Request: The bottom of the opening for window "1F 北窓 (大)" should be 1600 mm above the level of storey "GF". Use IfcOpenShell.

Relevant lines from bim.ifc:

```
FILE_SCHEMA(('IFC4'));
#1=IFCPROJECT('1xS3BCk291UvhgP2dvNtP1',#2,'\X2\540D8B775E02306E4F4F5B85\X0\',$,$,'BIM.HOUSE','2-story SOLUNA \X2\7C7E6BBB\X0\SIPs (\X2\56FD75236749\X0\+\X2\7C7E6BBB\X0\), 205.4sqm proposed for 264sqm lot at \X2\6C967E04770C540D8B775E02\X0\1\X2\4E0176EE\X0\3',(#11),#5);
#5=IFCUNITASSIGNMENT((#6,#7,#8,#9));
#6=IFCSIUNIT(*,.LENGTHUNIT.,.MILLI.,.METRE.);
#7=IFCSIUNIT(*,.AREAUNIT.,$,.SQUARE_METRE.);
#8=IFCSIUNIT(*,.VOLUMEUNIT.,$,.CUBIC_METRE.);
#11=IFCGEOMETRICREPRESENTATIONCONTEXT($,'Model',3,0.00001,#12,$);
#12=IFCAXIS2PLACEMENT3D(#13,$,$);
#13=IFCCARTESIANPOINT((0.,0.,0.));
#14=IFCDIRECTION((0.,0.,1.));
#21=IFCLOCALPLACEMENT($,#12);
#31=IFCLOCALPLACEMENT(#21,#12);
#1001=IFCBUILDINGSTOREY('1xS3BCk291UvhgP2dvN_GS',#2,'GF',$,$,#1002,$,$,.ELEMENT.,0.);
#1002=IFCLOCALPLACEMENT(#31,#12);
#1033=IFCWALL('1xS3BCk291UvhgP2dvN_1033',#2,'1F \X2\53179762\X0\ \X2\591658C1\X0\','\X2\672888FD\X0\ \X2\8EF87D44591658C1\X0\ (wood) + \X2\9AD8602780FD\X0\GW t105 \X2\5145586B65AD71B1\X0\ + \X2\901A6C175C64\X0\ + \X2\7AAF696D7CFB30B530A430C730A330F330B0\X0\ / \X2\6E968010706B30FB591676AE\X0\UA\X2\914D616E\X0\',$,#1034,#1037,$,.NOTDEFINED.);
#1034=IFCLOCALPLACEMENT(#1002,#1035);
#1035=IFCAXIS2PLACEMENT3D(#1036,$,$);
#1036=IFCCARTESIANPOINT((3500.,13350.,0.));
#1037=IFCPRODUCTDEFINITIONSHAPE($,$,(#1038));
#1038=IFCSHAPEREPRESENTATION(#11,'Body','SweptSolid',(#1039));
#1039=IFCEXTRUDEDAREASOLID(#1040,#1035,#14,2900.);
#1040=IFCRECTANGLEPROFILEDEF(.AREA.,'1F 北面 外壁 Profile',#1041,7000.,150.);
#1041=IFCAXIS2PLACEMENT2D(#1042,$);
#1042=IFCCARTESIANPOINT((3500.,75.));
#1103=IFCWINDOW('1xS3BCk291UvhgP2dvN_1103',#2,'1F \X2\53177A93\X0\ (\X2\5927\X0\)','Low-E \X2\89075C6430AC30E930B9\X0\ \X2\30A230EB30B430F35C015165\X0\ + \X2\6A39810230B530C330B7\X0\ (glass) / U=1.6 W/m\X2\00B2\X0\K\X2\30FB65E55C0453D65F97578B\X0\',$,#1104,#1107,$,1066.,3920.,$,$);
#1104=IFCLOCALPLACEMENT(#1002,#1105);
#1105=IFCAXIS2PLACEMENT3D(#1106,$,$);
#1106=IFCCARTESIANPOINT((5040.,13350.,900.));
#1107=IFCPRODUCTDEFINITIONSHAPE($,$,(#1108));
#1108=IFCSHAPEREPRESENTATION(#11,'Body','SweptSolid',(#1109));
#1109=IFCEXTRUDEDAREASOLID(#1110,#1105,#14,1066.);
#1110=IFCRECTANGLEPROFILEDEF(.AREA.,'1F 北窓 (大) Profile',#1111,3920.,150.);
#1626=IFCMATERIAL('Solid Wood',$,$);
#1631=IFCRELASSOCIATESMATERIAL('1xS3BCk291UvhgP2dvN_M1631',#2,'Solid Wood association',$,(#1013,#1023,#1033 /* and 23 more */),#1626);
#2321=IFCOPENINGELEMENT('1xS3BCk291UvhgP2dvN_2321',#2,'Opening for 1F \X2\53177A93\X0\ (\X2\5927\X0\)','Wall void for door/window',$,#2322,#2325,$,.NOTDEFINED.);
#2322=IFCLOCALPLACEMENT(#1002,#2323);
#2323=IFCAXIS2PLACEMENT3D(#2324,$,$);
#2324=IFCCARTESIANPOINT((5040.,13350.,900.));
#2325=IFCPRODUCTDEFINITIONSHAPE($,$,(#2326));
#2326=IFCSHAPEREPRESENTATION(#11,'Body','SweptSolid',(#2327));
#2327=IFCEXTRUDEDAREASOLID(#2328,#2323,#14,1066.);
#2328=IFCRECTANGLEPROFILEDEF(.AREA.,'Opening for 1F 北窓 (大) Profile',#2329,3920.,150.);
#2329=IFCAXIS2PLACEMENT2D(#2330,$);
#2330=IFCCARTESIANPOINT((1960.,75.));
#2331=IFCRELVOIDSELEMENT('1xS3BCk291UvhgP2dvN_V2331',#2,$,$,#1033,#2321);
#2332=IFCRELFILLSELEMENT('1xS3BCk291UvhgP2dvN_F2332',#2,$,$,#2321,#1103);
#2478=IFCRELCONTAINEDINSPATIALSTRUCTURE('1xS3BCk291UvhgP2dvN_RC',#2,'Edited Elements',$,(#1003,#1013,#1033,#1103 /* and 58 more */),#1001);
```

```python
import numpy as np
import ifcopenshell
import ifcopenshell.api.geometry
import ifcopenshell.geom
import ifcopenshell.util.element
import ifcopenshell.util.placement
import ifcopenshell.util.shape
import ifcopenshell.util.unit

model = ifcopenshell.open("bim.ifc")
unit_scale = ifcopenshell.util.unit.calculate_unit_scale(model)

window = model.by_guid("1xS3BCk291UvhgP2dvN_1103")
opening = window.FillsVoids[0].RelatingOpeningElement
storey = ifcopenshell.util.element.get_container(window, ifc_class="IfcBuildingStorey")
level = ifcopenshell.util.placement.get_local_placement(storey.ObjectPlacement)[2, 3]

# The opening's origin need not be at the sill, so measure its lowest point.
shape = ifcopenshell.geom.create_shape(ifcopenshell.geom.settings(), opening)
bottom = ifcopenshell.util.shape.get_shape_bottom_elevation(shape, shape.geometry) / unit_scale
dz = level + 1.6 / unit_scale - bottom

shift = np.array([0.0, 0.0, dz])
# The window is not placed relative to its opening, so move both.
for product in (opening, window):
    matrix = ifcopenshell.util.placement.get_local_placement(product.ObjectPlacement)
    matrix[:3, 3] += shift
    ifcopenshell.api.geometry.edit_object_placement(model, product=product, matrix=matrix, is_si=False)

print(f"moved by {dz * unit_scale:+.3f} m")

model.write("bim_edited.ifc")
```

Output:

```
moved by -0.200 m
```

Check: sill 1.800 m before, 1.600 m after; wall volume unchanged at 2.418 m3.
